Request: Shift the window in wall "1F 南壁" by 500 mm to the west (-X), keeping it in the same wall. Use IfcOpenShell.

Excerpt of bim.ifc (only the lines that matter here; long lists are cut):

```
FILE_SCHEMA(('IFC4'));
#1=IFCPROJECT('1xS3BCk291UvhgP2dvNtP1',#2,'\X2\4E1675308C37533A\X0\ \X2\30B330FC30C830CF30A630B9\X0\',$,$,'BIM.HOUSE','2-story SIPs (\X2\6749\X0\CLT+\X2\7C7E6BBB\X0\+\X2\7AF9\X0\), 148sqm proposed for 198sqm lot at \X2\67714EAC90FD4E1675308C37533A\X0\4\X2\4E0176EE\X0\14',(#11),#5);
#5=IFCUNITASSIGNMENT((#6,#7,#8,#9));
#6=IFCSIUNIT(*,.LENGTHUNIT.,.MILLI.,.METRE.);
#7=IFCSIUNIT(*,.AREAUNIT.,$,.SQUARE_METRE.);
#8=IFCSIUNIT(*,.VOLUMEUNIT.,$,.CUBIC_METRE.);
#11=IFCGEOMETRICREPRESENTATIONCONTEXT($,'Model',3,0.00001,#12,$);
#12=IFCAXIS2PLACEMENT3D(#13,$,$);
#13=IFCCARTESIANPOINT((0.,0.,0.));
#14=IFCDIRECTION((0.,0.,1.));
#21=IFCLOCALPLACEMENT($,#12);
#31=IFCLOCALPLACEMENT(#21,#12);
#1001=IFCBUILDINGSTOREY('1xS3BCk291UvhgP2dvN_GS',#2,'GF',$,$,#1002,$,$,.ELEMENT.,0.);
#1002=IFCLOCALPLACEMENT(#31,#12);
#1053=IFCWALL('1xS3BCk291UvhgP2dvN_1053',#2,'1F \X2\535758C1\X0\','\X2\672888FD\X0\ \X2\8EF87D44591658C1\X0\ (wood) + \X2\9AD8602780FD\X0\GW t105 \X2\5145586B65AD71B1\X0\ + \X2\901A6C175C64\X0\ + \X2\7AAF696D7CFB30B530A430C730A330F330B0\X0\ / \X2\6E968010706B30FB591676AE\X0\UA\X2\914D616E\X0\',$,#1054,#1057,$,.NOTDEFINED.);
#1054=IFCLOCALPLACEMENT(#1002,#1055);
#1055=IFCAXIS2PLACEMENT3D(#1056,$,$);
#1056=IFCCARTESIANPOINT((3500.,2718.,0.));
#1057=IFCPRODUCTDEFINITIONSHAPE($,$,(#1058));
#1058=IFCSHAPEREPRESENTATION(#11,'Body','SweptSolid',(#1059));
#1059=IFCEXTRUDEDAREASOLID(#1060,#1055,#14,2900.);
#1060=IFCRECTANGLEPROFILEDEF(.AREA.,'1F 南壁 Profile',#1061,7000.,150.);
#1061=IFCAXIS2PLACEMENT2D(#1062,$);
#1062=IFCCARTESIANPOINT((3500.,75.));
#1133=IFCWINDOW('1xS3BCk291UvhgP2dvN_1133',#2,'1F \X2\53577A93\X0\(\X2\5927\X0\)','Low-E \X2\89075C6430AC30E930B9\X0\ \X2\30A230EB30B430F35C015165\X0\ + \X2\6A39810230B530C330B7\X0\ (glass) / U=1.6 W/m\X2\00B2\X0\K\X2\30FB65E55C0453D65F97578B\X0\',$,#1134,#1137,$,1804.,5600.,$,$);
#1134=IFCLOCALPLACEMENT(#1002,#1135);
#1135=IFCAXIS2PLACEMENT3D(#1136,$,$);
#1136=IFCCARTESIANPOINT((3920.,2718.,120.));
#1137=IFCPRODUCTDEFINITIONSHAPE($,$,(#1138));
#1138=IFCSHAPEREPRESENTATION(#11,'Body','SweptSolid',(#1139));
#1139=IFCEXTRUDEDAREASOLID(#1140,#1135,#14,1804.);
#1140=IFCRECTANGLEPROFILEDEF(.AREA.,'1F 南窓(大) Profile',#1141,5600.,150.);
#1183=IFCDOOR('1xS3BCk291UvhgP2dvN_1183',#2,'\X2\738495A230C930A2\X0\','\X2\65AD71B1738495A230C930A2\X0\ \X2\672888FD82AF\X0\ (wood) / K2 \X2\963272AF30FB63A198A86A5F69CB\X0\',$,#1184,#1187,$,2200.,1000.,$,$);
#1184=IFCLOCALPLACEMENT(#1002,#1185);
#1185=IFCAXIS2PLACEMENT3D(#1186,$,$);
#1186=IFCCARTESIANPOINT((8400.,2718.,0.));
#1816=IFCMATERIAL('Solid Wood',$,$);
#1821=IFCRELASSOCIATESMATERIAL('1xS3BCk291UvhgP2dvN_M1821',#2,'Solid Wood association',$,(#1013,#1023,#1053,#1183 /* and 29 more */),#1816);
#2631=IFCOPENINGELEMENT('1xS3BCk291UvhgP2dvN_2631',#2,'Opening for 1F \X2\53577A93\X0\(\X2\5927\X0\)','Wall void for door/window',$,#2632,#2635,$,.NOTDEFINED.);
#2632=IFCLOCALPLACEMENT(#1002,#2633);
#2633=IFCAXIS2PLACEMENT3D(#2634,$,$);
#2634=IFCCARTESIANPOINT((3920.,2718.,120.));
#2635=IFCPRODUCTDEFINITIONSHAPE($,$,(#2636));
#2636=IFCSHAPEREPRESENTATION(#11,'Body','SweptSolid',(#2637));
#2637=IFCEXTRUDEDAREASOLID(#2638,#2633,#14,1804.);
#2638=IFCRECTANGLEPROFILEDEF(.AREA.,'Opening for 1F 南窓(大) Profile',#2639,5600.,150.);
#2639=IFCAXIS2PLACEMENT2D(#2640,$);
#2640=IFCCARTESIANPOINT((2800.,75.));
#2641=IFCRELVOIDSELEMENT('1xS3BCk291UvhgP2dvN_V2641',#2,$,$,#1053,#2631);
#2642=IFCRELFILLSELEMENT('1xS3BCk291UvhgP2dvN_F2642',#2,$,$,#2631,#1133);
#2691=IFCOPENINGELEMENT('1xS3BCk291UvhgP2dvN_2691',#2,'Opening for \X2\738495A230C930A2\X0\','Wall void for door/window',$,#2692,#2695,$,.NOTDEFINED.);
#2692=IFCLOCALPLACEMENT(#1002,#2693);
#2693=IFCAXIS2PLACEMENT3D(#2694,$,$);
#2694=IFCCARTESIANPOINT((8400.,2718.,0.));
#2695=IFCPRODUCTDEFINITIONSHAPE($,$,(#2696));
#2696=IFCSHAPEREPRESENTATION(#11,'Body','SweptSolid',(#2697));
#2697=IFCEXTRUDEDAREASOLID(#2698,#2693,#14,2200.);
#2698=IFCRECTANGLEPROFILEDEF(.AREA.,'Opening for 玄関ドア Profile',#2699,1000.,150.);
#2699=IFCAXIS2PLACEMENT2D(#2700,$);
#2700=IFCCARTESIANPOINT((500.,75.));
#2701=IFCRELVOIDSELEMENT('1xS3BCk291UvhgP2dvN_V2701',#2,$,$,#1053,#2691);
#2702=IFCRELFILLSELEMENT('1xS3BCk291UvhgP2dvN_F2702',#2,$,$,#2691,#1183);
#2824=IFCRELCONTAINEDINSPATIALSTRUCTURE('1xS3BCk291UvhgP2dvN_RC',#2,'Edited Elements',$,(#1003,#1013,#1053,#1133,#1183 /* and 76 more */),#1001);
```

```python
import ifcopenshell
import ifcopenshell.api.geometry
import ifcopenshell.util.placement

model = ifcopenshell.open("bim.ifc")

window = model.by_guid("1xS3BCk291UvhgP2dvN_1133")
opening = window.FillsVoids[0].RelatingOpeningElement
wall = opening.VoidsElements[0].RelatingBuildingElement

wall_matrix = ifcopenshell.util.placement.get_local_placement(wall.ObjectPlacement)
shift = wall_matrix[:3, 0] * -500.0
before = ifcopenshell.util.placement.get_local_placement(window.ObjectPlacement)[:3, 3].copy()

# The window is not placed relative to its opening, so move both.
for product in (opening, window):
    matrix = ifcopenshell.util.placement.get_local_placement(product.ObjectPlacement)
    matrix[:3, 3] += shift
    ifcopenshell.api.geometry.edit_object_placement(model, product=product, matrix=matrix, is_si=False)

after = ifcopenshell.util.placement.get_local_placement(window.ObjectPlacement)[:3, 3]
print("window moved by", (after - before).round(3) + 0.0)

model.write("bim_rev.ifc")
```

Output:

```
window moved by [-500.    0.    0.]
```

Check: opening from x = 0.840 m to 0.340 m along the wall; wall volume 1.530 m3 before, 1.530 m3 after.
